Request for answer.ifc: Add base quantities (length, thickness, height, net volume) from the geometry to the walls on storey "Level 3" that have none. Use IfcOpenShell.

First a look at what the model holds.

```python
import ifcopenshell
import ifcopenshell.util.element
import ifcopenshell.util.unit

model = ifcopenshell.open("answer.ifc")
print(model.schema)
for unit_type in ("LENGTHUNIT", "AREAUNIT", "VOLUMEUNIT"):
    print(unit_type, ifcopenshell.util.unit.calculate_unit_scale(model, unit_type))
storey = next(s for s in model.by_type("IfcBuildingStorey") if s.Name == "Level 3")
walls = [e for e in ifcopenshell.util.element.get_decomposition(storey) if e.is_a("IfcWall")]
for e in sorted(walls, key=lambda e: e.id()):
    print(e.id(), e.is_a(), e.Name, list(ifcopenshell.util.element.get_psets(e, qtos_only=True)), sep=" | ")
```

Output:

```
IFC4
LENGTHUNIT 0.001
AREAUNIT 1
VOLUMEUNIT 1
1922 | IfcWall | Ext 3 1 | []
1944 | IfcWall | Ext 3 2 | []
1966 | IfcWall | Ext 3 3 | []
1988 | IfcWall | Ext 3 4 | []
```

```python
import ifcopenshell
import ifcopenshell.api.pset
import ifcopenshell.geom
import ifcopenshell.util.element
import ifcopenshell.util.shape
import ifcopenshell.util.unit

model = ifcopenshell.open("answer.ifc")
unit_scale = ifcopenshell.util.unit.calculate_unit_scale(model)
volume_scale = ifcopenshell.util.unit.calculate_unit_scale(model, "VOLUMEUNIT")
settings = ifcopenshell.geom.settings()

storey = next(s for s in model.by_type("IfcBuildingStorey") if s.Name == "Level 3")
walls = [e for e in ifcopenshell.util.element.get_decomposition(storey) if e.is_a("IfcWall")]

for e in sorted(walls, key=lambda e: e.id()):
    if ifcopenshell.util.element.get_psets(e, qtos_only=True, should_inherit=False):
        continue
    # Geometry comes back in metres, in the element's own axes.
    shape = ifcopenshell.geom.create_shape(settings, e)
    values = {
        "Length": ifcopenshell.util.shape.get_x(shape.geometry) / unit_scale,
        "Width": ifcopenshell.util.shape.get_y(shape.geometry) / unit_scale,
        "Height": ifcopenshell.util.shape.get_z(shape.geometry) / unit_scale,
        "NetVolume": ifcopenshell.util.shape.get_volume(shape.geometry) / volume_scale,
    }
    qto = ifcopenshell.api.pset.add_qto(model, product=e, name="Qto_WallBaseQuantities")
    ifcopenshell.api.pset.edit_qto(model, qto=qto, properties=values)
    print(e.id(), {k: round(v, 3) for k, v in values.items()})

model.write("answer_edited.ifc")
```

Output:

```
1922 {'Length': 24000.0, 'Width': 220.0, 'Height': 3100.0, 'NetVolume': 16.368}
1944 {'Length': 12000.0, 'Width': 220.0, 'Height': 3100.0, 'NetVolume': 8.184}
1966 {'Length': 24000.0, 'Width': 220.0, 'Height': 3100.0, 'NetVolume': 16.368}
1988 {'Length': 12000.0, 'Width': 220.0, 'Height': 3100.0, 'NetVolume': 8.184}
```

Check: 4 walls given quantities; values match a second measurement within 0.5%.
